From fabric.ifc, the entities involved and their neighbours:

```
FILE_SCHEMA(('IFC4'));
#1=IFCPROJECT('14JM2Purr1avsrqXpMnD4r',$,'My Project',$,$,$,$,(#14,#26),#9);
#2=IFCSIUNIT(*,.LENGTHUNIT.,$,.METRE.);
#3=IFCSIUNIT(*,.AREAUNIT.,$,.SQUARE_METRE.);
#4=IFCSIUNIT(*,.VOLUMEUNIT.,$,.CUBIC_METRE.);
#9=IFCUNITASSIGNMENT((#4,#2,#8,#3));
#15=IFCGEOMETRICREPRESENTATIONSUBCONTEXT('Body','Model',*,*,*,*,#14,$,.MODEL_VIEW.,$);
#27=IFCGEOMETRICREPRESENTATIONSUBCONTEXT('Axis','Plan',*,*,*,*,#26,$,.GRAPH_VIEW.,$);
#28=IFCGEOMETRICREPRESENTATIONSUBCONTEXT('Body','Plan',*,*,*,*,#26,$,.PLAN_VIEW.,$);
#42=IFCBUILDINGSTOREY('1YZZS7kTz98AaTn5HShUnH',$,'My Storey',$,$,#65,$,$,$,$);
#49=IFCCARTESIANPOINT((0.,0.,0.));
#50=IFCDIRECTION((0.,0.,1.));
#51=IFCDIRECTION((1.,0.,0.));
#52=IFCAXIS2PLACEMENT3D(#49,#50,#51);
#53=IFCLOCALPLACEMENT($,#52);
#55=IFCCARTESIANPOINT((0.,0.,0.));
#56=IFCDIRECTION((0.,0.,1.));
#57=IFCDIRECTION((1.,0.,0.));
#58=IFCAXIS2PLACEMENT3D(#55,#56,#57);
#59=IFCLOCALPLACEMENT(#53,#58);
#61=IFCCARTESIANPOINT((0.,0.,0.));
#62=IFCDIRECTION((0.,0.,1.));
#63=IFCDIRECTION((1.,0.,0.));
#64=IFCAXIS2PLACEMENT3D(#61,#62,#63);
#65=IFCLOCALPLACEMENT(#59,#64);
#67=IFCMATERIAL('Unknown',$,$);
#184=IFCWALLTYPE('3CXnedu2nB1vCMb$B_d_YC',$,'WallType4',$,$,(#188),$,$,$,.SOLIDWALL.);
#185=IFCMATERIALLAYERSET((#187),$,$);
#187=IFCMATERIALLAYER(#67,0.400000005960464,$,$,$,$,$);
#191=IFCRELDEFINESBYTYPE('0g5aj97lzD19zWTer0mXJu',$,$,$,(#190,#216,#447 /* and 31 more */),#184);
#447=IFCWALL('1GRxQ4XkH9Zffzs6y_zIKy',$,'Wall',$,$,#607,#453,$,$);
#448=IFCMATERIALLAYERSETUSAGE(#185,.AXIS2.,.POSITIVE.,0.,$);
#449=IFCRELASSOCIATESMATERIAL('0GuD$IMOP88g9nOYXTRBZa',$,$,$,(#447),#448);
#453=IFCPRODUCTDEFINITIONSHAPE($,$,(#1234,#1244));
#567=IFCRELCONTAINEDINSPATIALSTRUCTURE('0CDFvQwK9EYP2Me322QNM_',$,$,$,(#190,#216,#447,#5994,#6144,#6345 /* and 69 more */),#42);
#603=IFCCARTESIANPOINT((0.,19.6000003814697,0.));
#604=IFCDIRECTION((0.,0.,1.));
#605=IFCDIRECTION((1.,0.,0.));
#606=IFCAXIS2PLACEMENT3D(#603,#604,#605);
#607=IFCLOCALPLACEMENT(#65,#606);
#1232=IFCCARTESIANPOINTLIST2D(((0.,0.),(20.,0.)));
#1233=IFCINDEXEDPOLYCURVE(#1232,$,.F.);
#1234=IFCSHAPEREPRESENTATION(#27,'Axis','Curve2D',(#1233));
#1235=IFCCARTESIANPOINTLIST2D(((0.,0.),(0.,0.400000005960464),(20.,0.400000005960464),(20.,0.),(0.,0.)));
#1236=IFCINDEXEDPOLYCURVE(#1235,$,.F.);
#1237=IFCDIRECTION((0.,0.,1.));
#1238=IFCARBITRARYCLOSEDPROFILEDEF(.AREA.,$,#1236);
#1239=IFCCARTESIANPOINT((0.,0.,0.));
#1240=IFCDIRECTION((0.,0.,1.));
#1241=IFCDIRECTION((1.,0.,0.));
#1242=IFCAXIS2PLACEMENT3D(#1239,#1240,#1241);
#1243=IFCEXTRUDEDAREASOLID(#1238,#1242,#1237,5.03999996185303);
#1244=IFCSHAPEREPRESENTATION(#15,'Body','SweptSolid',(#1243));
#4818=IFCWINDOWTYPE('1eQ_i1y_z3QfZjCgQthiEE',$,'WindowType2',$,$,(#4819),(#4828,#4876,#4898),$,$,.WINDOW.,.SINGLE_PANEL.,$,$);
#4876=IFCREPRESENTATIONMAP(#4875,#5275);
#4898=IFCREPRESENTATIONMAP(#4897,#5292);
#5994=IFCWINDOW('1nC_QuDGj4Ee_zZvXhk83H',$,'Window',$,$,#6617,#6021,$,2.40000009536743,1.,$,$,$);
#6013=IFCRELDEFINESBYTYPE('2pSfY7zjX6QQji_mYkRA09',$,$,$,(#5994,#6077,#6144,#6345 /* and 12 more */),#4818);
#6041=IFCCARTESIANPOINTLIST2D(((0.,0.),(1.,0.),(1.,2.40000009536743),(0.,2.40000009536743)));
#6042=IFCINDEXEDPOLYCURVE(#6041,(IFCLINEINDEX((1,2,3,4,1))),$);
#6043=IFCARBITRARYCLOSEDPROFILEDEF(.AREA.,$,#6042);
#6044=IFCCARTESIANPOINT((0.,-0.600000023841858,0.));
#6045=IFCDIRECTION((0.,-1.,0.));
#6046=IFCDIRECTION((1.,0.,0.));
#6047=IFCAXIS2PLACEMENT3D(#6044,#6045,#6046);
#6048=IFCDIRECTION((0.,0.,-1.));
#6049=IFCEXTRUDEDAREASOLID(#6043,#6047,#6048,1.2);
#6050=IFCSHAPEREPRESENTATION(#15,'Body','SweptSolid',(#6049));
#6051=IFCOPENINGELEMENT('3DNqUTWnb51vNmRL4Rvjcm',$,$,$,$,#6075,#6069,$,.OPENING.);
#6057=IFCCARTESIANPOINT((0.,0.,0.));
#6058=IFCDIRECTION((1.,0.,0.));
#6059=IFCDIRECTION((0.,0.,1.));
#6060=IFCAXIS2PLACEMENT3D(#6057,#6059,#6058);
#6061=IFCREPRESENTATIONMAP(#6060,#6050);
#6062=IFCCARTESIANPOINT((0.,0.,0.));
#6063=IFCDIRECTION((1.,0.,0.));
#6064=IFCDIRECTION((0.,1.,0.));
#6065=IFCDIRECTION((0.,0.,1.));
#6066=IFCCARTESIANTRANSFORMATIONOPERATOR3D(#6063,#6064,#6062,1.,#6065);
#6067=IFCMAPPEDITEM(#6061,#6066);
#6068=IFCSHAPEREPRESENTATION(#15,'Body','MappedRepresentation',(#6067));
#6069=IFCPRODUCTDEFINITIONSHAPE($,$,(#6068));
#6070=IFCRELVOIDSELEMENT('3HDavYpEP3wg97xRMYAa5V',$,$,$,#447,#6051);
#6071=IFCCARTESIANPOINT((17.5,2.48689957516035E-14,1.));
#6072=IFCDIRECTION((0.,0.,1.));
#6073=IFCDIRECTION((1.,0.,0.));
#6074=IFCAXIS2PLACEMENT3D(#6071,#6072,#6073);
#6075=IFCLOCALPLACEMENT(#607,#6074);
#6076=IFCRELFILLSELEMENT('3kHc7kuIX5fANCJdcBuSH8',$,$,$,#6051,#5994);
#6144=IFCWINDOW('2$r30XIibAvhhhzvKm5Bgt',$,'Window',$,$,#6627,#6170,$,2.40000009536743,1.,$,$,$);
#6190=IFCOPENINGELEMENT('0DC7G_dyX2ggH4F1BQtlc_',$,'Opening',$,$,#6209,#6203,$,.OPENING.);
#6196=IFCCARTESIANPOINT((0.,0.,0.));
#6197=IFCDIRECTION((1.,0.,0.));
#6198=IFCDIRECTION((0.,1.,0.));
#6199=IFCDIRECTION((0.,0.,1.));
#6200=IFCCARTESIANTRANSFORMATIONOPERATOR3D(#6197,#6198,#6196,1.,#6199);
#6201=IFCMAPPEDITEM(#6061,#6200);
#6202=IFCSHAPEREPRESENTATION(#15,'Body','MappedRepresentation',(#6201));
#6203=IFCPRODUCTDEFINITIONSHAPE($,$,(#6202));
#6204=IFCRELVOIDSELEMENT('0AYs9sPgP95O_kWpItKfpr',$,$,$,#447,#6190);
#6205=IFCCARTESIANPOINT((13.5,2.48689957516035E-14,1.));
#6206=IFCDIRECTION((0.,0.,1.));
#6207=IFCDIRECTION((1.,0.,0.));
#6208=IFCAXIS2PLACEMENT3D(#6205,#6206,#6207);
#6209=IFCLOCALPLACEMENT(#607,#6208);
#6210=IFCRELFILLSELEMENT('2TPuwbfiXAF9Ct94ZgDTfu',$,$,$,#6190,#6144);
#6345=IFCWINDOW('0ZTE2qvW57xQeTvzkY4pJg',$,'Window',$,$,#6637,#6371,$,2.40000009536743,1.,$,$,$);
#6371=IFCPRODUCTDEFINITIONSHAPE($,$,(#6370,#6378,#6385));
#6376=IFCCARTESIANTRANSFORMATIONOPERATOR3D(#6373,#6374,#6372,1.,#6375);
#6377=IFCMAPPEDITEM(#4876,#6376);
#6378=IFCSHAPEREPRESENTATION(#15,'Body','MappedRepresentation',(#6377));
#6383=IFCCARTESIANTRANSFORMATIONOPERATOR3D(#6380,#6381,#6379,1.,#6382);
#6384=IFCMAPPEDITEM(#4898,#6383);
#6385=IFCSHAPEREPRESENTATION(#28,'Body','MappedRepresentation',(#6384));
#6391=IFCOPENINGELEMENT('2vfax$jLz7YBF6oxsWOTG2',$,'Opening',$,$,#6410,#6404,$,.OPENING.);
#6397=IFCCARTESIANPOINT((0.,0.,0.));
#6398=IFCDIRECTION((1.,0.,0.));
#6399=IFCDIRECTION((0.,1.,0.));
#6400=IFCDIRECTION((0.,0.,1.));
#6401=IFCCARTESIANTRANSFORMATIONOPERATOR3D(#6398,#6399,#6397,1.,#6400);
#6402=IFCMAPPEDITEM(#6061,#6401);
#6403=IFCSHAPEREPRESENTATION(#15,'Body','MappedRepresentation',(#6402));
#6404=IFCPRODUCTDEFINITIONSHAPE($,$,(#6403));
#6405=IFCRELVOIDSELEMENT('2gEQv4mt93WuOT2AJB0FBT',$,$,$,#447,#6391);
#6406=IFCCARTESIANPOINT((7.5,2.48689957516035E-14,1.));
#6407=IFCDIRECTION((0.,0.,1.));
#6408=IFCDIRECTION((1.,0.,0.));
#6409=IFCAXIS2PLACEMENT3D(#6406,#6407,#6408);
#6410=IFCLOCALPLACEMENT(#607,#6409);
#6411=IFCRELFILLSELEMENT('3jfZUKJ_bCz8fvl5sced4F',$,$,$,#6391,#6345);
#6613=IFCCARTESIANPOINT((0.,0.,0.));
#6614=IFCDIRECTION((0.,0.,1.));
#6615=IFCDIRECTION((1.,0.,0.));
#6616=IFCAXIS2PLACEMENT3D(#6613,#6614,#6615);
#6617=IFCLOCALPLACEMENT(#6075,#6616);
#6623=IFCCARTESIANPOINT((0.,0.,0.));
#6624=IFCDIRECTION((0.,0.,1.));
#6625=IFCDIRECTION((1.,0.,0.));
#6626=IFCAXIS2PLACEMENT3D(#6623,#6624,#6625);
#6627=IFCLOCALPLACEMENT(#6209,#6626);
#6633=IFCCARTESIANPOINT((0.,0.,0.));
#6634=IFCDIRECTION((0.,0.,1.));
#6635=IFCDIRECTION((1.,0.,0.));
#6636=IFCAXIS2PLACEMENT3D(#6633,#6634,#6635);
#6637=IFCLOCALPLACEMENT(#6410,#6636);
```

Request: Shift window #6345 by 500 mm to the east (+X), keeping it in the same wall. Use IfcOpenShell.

```python
import ifcopenshell
import ifcopenshell.api.geometry
import ifcopenshell.util.placement
import ifcopenshell.util.unit

model = ifcopenshell.open("fabric.ifc")
unit_scale = ifcopenshell.util.unit.calculate_unit_scale(model)

window = model.by_guid("0ZTE2qvW57xQeTvzkY4pJg")
opening = window.FillsVoids[0].RelatingOpeningElement
wall = opening.VoidsElements[0].RelatingBuildingElement

wall_matrix = ifcopenshell.util.placement.get_local_placement(wall.ObjectPlacement)
shift = wall_matrix[:3, 0] * 0.5 / unit_scale
before = ifcopenshell.util.placement.get_local_placement(window.ObjectPlacement)[:3, 3].copy()

# The window is placed relative to its opening, so it follows when the opening moves.
matrix = ifcopenshell.util.placement.get_local_placement(opening.ObjectPlacement)
matrix[:3, 3] += shift
ifcopenshell.api.geometry.edit_object_placement(
    model, product=opening, matrix=matrix, is_si=False, should_transform_children=True
)

after = ifcopenshell.util.placement.get_local_placement(window.ObjectPlacement)[:3, 3]
print("window moved by", (after - before).round(3) + 0.0)

model.write("fabric_v2.ifc")
```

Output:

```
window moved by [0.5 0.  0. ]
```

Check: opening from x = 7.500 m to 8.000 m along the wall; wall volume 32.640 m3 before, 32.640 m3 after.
